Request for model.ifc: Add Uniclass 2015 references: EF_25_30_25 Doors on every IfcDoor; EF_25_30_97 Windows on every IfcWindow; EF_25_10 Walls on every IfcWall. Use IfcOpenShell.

First a look at what the model holds.

```python
import ifcopenshell

model = ifcopenshell.open("model.ifc")
print(model.schema)
print("classifications:", [c.Name for c in model.by_type("IfcClassification")])
for ifc_class in ("IfcDoor", "IfcRoof", "IfcStair", "IfcWall", "IfcWindow"):
    print(ifc_class, len(model.by_type(ifc_class)))
```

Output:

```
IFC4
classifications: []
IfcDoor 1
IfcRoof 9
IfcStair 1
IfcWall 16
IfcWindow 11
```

```python
import ifcopenshell
import ifcopenshell.api.classification

model = ifcopenshell.open("model.ifc")

system = ifcopenshell.api.classification.add_classification(model, classification="Uniclass 2015")

codes = {
    "IfcDoor": ("EF_25_30_25", "Doors"),
    "IfcWindow": ("EF_25_30_97", "Windows"),
    "IfcWall": ("EF_25_10", "Walls"),
}
for ifc_class, (code, name) in codes.items():
    products = model.by_type(ifc_class)
    ifcopenshell.api.classification.add_reference(
        model, products=products, classification=system, identification=code, name=name
    )
    print(code, len(products))

model.write("model_edited.ifc")
```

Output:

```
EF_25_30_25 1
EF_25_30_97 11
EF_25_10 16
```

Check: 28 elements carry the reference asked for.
